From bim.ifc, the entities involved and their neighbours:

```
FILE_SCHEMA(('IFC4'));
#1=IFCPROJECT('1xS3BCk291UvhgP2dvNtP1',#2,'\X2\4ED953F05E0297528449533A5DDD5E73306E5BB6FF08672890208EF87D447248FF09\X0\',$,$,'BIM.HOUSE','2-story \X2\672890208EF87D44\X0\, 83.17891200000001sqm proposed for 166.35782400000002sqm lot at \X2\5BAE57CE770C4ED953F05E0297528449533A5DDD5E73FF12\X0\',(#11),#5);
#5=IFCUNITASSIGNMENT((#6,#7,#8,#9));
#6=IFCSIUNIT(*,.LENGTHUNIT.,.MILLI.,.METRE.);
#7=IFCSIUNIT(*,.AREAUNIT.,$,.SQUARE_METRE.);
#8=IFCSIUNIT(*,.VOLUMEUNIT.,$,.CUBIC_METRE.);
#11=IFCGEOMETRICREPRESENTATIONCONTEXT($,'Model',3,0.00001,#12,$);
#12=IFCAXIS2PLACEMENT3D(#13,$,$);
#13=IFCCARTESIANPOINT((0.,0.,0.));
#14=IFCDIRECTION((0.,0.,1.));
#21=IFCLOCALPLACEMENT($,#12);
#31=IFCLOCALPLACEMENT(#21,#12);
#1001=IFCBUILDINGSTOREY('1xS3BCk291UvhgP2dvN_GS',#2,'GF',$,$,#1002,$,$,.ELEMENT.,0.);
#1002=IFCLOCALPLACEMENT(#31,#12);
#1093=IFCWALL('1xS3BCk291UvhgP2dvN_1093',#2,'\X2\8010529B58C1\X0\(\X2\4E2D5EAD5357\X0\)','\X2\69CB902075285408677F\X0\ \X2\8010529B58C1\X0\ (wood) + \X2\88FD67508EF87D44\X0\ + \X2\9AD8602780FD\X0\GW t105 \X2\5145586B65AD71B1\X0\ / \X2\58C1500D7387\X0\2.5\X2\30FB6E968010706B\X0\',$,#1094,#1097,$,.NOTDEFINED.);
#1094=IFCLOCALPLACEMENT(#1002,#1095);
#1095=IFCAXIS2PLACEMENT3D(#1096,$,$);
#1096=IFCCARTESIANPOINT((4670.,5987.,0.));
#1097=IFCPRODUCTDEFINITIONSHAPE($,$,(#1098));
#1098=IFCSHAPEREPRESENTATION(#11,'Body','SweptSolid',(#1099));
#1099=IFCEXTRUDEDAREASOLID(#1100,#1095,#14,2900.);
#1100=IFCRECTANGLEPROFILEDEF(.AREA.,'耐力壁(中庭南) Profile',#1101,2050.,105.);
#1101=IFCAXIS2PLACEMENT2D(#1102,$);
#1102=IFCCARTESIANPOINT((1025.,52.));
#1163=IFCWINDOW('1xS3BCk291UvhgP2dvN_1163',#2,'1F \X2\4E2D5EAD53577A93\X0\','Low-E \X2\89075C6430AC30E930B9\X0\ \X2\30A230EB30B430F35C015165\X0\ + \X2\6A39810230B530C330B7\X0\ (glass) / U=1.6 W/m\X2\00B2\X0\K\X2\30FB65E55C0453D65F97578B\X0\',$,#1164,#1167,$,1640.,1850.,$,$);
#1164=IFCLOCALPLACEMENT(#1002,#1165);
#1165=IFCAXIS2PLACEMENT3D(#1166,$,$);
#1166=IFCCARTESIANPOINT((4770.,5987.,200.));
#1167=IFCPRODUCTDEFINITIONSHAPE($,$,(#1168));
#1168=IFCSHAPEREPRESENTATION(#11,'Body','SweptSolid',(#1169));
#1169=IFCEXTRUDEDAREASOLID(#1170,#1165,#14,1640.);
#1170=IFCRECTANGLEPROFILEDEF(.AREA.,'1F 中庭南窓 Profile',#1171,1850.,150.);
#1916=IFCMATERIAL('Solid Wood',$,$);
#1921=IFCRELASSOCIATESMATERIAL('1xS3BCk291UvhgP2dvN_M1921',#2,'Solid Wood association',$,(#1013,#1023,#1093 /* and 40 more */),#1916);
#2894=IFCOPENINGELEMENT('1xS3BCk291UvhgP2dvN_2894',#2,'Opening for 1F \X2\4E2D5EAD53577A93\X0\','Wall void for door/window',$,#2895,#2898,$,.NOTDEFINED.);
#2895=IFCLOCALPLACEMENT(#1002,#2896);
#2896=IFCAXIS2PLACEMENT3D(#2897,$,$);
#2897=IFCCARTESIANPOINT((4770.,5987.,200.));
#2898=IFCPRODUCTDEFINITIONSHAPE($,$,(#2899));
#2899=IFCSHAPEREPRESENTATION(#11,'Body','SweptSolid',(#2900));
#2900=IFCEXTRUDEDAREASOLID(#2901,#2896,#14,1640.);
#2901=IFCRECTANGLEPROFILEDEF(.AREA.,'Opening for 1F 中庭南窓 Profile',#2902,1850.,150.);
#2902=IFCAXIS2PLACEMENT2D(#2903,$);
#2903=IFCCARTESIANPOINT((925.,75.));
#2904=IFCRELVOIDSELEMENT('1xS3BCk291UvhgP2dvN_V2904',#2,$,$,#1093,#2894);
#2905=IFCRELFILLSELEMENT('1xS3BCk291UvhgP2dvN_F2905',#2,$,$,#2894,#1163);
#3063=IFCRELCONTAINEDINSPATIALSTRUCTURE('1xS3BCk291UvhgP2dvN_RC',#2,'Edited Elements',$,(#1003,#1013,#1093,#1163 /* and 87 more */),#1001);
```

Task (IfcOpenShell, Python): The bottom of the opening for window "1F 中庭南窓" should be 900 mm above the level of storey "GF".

```python
import numpy as np
import ifcopenshell
import ifcopenshell.api.geometry
import ifcopenshell.geom
import ifcopenshell.util.element
import ifcopenshell.util.placement
import ifcopenshell.util.shape
import ifcopenshell.util.unit

model = ifcopenshell.open("bim.ifc")
unit_scale = ifcopenshell.util.unit.calculate_unit_scale(model)

window = model.by_guid("1xS3BCk291UvhgP2dvN_1163")
opening = window.FillsVoids[0].RelatingOpeningElement
storey = ifcopenshell.util.element.get_container(window, ifc_class="IfcBuildingStorey")
level = ifcopenshell.util.placement.get_local_placement(storey.ObjectPlacement)[2, 3]

# The opening's origin need not be at the sill, so measure its lowest point.
shape = ifcopenshell.geom.create_shape(ifcopenshell.geom.settings(), opening)
bottom = ifcopenshell.util.shape.get_shape_bottom_elevation(shape, shape.geometry) / unit_scale
dz = level + 0.9 / unit_scale - bottom

shift = np.array([0.0, 0.0, dz])
# The window is not placed relative to its opening, so move both.
for product in (opening, window):
    matrix = ifcopenshell.util.placement.get_local_placement(product.ObjectPlacement)
    matrix[:3, 3] += shift
    ifcopenshell.api.geometry.edit_object_placement(model, product=product, matrix=matrix, is_si=False)

print(f"moved by {dz * unit_scale:+.3f} m")

model.write("bim-out.ifc")
```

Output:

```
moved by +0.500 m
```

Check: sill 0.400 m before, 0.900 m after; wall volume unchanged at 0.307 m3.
